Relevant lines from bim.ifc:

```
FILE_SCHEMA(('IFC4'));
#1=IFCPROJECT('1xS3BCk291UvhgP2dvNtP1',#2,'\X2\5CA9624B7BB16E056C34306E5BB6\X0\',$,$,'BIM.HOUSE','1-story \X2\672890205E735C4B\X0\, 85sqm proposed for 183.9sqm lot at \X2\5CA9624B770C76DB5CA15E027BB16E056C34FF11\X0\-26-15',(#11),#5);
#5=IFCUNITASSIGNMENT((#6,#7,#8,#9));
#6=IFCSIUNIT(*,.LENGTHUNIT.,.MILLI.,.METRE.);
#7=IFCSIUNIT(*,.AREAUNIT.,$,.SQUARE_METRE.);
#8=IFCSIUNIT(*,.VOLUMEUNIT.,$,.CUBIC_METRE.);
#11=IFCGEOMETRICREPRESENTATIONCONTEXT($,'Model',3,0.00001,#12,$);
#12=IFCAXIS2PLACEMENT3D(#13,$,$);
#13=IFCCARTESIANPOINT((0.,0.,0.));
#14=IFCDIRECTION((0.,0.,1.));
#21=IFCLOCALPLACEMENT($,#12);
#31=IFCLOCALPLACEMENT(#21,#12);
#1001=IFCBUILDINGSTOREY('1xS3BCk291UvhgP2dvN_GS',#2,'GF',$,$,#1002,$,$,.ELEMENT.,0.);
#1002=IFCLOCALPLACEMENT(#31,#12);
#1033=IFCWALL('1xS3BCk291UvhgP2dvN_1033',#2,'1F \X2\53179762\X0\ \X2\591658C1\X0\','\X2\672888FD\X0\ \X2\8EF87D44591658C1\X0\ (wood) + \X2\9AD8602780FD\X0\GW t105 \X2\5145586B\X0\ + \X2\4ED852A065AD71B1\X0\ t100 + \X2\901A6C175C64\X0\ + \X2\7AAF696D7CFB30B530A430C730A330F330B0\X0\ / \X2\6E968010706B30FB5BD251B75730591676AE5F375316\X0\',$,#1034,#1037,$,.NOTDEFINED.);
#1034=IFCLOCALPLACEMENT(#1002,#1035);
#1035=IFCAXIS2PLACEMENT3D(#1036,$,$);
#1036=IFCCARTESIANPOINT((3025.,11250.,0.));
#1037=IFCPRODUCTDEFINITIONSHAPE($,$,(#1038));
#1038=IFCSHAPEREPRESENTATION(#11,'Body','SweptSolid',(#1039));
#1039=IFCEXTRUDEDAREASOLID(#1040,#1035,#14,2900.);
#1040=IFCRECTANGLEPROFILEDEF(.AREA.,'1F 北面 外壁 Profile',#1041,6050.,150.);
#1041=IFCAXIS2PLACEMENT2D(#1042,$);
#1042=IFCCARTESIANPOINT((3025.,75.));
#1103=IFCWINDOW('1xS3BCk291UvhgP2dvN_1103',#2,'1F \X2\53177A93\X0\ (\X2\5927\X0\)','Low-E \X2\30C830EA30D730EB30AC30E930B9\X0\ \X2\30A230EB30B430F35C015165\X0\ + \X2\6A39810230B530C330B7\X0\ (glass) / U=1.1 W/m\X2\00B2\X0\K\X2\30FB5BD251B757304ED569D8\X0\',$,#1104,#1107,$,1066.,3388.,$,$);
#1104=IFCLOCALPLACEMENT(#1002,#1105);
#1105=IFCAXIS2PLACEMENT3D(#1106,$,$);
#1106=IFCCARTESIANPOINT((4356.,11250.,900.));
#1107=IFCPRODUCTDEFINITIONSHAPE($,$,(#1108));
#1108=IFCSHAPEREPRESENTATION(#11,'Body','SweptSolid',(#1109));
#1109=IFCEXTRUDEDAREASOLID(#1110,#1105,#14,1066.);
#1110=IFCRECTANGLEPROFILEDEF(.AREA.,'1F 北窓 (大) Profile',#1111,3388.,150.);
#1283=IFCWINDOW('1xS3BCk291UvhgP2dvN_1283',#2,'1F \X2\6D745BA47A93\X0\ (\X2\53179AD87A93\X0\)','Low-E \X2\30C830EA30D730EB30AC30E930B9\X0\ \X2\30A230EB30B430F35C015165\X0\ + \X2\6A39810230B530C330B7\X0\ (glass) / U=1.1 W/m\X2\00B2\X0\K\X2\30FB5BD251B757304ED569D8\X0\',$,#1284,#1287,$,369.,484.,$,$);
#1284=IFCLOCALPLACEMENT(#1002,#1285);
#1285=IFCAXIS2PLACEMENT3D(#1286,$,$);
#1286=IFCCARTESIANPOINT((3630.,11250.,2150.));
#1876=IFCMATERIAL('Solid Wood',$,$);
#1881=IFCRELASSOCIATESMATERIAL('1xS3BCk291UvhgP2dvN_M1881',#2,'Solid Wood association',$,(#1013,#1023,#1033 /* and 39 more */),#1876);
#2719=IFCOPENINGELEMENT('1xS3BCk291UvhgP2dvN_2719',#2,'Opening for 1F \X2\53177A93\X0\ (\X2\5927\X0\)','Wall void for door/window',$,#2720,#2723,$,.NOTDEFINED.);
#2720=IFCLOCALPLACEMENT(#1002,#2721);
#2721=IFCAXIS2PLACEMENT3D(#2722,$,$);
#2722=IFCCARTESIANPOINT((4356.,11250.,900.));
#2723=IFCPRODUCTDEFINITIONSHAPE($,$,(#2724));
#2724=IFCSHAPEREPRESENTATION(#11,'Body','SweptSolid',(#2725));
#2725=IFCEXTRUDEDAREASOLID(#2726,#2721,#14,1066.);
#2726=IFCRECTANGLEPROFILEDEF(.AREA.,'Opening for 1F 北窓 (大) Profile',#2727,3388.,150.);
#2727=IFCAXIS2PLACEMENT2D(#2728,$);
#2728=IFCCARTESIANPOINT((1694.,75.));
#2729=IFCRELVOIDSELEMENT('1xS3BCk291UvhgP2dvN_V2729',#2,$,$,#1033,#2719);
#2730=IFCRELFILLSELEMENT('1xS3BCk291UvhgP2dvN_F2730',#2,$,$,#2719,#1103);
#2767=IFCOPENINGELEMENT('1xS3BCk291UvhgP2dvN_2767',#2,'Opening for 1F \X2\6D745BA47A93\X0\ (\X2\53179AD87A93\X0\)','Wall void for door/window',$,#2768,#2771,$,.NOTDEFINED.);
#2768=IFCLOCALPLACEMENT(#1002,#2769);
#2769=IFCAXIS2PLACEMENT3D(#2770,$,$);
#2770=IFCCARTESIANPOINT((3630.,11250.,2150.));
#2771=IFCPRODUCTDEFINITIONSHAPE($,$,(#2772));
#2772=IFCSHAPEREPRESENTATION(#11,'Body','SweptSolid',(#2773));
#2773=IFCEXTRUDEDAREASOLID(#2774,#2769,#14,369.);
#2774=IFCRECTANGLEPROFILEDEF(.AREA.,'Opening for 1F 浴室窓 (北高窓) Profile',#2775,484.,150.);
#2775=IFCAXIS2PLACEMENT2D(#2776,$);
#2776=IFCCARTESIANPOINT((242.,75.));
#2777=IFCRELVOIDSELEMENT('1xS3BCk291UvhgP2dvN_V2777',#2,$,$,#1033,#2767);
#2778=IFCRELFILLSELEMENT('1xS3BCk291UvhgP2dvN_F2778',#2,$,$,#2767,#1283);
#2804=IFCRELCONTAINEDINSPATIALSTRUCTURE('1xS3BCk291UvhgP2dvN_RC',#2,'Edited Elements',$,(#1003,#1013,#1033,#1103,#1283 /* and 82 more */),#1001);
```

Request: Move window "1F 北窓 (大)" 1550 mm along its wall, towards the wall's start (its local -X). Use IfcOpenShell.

```python
import ifcopenshell
import ifcopenshell.api.geometry
import ifcopenshell.util.placement

model = ifcopenshell.open("bim.ifc")

window = model.by_guid("1xS3BCk291UvhgP2dvN_1103")
opening = window.FillsVoids[0].RelatingOpeningElement
wall = opening.VoidsElements[0].RelatingBuildingElement

wall_matrix = ifcopenshell.util.placement.get_local_placement(wall.ObjectPlacement)
shift = wall_matrix[:3, 0] * -1550.0
before = ifcopenshell.util.placement.get_local_placement(window.ObjectPlacement)[:3, 3].copy()

# The window is not placed relative to its opening, so move both.
for product in (opening, window):
    matrix = ifcopenshell.util.placement.get_local_placement(product.ObjectPlacement)
    matrix[:3, 3] += shift
    ifcopenshell.api.geometry.edit_object_placement(model, product=product, matrix=matrix, is_si=False)

after = ifcopenshell.util.placement.get_local_placement(window.ObjectPlacement)[:3, 3]
print("window moved by", (after - before).round(3) + 0.0)

model.write("bim_edited.ifc")
```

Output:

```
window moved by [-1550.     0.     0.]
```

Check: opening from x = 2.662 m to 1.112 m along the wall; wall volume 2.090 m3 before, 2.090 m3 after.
